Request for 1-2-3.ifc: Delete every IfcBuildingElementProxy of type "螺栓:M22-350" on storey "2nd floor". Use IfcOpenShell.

First a look at what the model holds.

```python
import ifcopenshell
import ifcopenshell.util.element

model = ifcopenshell.open("1-2-3.ifc")
print(model.schema)
storey = next(s for s in model.by_type("IfcBuildingStorey") if s.Name == "2nd floor")
proxies = [e for e in ifcopenshell.util.element.get_decomposition(storey) if e.is_a("IfcBuildingElementProxy")]
seen = {}
for e in proxies:
    element_type = ifcopenshell.util.element.get_type(e)
    name = element_type.Name if element_type not in (None, e) else None
    seen[name] = seen.get(name, 0) + 1
for name, count in sorted(seen.items(), key=str):
    print(count, "x", name)
```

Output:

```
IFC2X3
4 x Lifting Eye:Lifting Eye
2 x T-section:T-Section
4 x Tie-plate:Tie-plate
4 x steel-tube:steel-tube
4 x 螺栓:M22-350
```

```python
import ifcopenshell
import ifcopenshell.api.root
import ifcopenshell.util.element

model = ifcopenshell.open("1-2-3.ifc")

storey = next(s for s in model.by_type("IfcBuildingStorey") if s.Name == "2nd floor")
proxies = [e for e in ifcopenshell.util.element.get_decomposition(storey) if e.is_a("IfcBuildingElementProxy")]
targets = [e for e in proxies if (t := ifcopenshell.util.element.get_type(e)) not in (None, e) and t.Name == "螺栓:M22-350"]

for e in targets:
    ifcopenshell.api.root.remove_product(model, product=e)
print(len(targets), "removed")

model.write("1-2-3_rev.ifc")
```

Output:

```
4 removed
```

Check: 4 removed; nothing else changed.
